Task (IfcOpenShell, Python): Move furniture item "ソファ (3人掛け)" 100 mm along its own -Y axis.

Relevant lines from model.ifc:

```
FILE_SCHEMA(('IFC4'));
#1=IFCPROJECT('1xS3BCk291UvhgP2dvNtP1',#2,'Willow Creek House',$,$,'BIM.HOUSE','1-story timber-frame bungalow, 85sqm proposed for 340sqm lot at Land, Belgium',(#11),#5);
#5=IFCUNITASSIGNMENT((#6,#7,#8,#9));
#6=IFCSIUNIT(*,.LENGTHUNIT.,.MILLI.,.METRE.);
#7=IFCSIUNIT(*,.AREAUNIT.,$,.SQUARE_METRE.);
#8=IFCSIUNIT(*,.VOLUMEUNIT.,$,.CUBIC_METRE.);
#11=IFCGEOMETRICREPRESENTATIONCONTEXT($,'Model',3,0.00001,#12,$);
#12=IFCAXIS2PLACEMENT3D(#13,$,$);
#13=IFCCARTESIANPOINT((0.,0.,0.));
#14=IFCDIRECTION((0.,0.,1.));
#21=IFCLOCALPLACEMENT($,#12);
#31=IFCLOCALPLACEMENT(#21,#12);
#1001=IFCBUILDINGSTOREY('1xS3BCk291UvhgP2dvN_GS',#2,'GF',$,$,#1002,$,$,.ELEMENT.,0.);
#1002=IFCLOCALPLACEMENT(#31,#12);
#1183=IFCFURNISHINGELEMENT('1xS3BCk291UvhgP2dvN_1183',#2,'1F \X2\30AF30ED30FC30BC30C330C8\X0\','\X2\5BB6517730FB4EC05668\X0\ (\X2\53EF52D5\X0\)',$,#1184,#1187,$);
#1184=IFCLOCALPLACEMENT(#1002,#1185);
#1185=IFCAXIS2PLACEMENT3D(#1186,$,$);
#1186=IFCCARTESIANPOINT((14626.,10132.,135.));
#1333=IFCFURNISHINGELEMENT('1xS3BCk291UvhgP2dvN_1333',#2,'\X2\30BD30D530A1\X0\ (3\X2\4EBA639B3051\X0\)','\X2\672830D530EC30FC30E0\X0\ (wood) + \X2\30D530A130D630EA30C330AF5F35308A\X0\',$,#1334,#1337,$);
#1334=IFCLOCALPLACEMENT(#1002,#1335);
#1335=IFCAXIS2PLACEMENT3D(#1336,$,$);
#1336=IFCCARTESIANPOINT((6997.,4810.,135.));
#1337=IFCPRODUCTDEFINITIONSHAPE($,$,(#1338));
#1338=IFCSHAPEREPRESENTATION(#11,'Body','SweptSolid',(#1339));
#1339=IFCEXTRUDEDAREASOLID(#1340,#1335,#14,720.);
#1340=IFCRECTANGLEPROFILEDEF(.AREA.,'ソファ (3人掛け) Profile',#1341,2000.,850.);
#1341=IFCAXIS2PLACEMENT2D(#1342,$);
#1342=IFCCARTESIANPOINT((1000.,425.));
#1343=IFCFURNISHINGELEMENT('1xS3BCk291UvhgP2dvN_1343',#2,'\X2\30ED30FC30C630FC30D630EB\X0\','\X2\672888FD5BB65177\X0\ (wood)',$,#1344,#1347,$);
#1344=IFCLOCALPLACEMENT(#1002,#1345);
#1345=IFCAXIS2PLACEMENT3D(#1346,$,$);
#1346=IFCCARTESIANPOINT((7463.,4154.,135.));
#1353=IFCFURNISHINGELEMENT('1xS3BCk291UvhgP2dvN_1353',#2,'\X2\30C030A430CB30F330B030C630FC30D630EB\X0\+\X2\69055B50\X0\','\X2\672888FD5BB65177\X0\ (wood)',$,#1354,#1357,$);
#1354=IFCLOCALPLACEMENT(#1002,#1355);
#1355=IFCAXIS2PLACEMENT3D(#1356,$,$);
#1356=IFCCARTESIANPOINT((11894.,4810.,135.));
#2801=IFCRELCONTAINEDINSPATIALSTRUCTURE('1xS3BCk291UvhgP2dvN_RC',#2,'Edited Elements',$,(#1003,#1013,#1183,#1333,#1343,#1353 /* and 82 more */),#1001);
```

```python
import ifcopenshell
import ifcopenshell.api.geometry
import ifcopenshell.util.placement

model = ifcopenshell.open("model.ifc")

item = model.by_id(1333)
matrix = ifcopenshell.util.placement.get_local_placement(item.ObjectPlacement)
matrix[:3, 3] -= matrix[:3, 1] * 100.0
ifcopenshell.api.geometry.edit_object_placement(model, product=item, matrix=matrix, is_si=False)

print(ifcopenshell.util.placement.get_local_placement(item.ObjectPlacement).round(3) + 0.0)

model.write("model_rev.ifc")
```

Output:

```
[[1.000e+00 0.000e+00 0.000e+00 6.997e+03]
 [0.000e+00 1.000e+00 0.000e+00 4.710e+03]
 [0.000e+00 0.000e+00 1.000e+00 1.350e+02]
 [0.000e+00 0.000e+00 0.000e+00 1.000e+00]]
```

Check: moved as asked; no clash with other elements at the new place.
